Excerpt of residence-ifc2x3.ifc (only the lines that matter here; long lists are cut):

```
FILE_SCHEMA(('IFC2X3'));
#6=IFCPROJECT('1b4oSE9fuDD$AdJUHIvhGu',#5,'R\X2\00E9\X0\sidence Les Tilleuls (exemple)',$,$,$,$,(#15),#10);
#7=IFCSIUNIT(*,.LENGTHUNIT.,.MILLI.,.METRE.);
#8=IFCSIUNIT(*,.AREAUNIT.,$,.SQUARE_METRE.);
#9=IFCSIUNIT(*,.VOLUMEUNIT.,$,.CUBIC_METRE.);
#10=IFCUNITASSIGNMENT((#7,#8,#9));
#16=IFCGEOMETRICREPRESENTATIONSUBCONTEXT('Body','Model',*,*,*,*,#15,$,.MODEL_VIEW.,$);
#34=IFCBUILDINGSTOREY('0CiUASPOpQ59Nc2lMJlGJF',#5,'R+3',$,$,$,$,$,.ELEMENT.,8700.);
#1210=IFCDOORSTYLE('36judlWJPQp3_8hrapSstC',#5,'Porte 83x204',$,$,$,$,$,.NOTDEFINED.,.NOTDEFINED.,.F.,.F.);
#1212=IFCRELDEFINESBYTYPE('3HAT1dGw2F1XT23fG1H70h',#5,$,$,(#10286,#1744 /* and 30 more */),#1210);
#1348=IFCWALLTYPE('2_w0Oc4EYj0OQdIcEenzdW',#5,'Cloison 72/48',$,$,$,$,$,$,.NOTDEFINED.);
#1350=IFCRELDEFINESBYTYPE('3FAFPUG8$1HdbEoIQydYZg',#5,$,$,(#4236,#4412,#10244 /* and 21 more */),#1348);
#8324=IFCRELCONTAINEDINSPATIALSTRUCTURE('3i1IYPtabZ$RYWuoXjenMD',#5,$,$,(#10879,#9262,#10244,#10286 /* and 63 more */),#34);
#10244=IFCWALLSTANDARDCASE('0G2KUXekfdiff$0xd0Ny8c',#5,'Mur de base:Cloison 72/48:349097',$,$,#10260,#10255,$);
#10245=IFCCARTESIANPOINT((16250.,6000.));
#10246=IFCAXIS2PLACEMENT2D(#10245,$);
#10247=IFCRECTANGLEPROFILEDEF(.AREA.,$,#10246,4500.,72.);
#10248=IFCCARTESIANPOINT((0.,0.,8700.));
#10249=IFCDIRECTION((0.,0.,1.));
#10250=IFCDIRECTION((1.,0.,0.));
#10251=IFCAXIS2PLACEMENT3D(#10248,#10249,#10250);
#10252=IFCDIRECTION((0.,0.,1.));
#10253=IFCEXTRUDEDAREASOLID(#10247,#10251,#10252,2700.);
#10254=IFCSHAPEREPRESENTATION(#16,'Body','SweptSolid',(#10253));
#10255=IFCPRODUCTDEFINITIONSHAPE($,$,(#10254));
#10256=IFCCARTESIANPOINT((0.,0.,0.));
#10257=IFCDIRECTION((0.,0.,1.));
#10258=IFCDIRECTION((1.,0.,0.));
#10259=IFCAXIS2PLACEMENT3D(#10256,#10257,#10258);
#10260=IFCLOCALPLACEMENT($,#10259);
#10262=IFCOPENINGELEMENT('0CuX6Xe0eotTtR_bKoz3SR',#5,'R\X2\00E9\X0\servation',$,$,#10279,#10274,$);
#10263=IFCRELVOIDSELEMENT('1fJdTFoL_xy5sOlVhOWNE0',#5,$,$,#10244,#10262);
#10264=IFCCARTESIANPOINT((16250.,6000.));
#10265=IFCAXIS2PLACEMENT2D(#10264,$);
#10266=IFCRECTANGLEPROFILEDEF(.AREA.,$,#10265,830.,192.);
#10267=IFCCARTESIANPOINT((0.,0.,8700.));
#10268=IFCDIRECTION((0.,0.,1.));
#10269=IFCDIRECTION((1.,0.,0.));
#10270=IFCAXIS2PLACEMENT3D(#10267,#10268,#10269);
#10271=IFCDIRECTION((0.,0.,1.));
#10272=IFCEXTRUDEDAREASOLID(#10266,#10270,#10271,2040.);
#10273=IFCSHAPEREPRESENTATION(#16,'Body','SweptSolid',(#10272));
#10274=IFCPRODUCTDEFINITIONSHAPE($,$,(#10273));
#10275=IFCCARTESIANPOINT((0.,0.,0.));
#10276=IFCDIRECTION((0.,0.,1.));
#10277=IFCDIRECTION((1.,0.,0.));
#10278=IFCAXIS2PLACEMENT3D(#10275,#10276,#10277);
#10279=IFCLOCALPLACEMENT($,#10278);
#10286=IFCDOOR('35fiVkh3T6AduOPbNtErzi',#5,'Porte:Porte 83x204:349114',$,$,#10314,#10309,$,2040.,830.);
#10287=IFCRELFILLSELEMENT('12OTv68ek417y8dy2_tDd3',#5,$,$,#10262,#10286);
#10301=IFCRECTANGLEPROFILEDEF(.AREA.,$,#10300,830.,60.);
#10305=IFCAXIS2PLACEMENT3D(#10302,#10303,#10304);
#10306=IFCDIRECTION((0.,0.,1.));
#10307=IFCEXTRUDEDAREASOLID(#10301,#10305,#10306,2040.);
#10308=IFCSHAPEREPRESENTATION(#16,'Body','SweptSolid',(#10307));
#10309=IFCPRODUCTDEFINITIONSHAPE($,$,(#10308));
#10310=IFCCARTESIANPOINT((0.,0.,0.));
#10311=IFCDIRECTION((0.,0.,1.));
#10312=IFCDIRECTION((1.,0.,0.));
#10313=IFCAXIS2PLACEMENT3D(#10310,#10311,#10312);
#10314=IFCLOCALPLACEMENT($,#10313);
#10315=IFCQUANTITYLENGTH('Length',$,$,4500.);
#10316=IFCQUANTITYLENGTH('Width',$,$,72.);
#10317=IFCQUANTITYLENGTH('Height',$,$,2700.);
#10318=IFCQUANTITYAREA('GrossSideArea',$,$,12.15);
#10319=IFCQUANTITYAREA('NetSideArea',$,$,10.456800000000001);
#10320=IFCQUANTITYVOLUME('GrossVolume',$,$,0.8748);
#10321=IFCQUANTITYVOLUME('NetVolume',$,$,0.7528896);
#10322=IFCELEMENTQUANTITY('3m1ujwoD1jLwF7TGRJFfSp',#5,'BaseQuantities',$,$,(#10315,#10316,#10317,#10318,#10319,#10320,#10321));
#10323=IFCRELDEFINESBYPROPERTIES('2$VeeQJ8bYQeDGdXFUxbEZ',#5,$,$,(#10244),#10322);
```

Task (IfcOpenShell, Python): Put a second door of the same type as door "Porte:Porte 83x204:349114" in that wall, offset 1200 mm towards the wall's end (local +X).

```python
import ifcopenshell
import ifcopenshell.api.feature
import ifcopenshell.api.geometry
import ifcopenshell.api.pset
import ifcopenshell.api.root
import ifcopenshell.geom
import ifcopenshell.util.element
import ifcopenshell.util.placement
import ifcopenshell.util.shape
import ifcopenshell.util.unit

model = ifcopenshell.open("residence-ifc2x3.ifc")
unit_scale = ifcopenshell.util.unit.calculate_unit_scale(model)
area_scale = ifcopenshell.util.unit.calculate_unit_scale(model, "AREAUNIT")
volume_scale = ifcopenshell.util.unit.calculate_unit_scale(model, "VOLUMEUNIT")
settings = ifcopenshell.geom.settings()


def volume(element):
    """Net volume in cubic metres, openings subtracted."""
    shape = ifcopenshell.geom.create_shape(settings, element)
    return ifcopenshell.util.shape.get_volume(shape.geometry)


def reuse_history(source, copy):
    """copy_class also copies each property set's owner history, people and application; keep the originals."""
    for rel in copy.IsDefinedBy:
        if rel.is_a("IfcRelDefinesByProperties") and (history := rel.RelatingPropertyDefinition.OwnerHistory):
            rel.RelatingPropertyDefinition.OwnerHistory = source.OwnerHistory
            ifcopenshell.util.element.remove_deep2(model, history)


door = model.by_guid("35fiVkh3T6AduOPbNtErzi")
opening = door.FillsVoids[0].RelatingOpeningElement
wall = opening.VoidsElements[0].RelatingBuildingElement
before = volume(wall)
shift = ifcopenshell.util.placement.get_local_placement(wall.ObjectPlacement)[:3, 0] * 1.2 / unit_scale

# copy_class copies the void relationship, type, container and properties, but no geometry.
new_opening = ifcopenshell.api.root.copy_class(model, product=opening)
new_opening.Representation = ifcopenshell.util.element.copy_deep(
    model, opening.Representation, exclude=["IfcGeometricRepresentationContext", "IfcRepresentationMap"]
)
reuse_history(opening, new_opening)
new_door = ifcopenshell.api.root.copy_class(model, product=door)
new_door.Representation = ifcopenshell.util.element.copy_deep(
    model, door.Representation, exclude=["IfcGeometricRepresentationContext", "IfcRepresentationMap"]
)
new_door.Name = "Porte:Porte 83x204"
reuse_history(door, new_door)
fills = ifcopenshell.api.feature.add_filling(model, opening=new_opening, element=new_door)
fills.OwnerHistory = new_door.OwnerHistory  # required in IFC2X3

for old, new in ((opening, new_opening), (door, new_door)):
    matrix = ifcopenshell.util.placement.get_local_placement(old.ObjectPlacement)
    matrix[:3, 3] += shift
    ifcopenshell.api.geometry.edit_object_placement(model, product=new, matrix=matrix, is_si=False)

after = volume(wall)
thickness = 0.072  # wall thickness in metres

# Update the wall's stored quantities.
qto = model.by_id(ifcopenshell.util.element.get_pset(wall, "BaseQuantities", should_inherit=False)["id"])
ifcopenshell.api.pset.edit_qto(model, qto=qto, properties={
    "NetSideArea": after / thickness / area_scale,
    "NetVolume": after / volume_scale,
})

print(f"wall volume {before:.3f} -> {after:.3f} m3")

model.write("residence-ifc2x3-out.ifc")
```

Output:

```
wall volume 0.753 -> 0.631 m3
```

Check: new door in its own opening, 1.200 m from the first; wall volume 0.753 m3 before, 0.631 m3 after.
